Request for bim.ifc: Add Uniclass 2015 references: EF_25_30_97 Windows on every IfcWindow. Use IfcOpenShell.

First a look at what the model holds.

```python
import ifcopenshell

model = ifcopenshell.open("bim.ifc")
print(model.schema)
print("classifications:", [c.Name for c in model.by_type("IfcClassification")])
for ifc_class in ("IfcDoor", "IfcRoof", "IfcStair", "IfcWall", "IfcWindow"):
    print(ifc_class, len(model.by_type(ifc_class)))
```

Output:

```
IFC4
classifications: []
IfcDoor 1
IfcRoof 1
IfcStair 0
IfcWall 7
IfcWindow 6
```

```python
import ifcopenshell
import ifcopenshell.api.classification

model = ifcopenshell.open("bim.ifc")

system = ifcopenshell.api.classification.add_classification(model, classification="Uniclass 2015")

codes = {
    "IfcWindow": ("EF_25_30_97", "Windows"),
}
for ifc_class, (code, name) in codes.items():
    products = model.by_type(ifc_class)
    ifcopenshell.api.classification.add_reference(
        model, products=products, classification=system, identification=code, name=name
    )
    print(code, len(products))

model.write("bim_rev.ifc")
```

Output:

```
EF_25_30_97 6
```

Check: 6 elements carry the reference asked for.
